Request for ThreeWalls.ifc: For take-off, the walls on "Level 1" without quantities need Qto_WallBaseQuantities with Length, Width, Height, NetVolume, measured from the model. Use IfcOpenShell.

First a look at what the model holds.

```python
import ifcopenshell
import ifcopenshell.util.element
import ifcopenshell.util.unit

model = ifcopenshell.open("ThreeWalls.ifc")
print(model.schema)
for unit_type in ("LENGTHUNIT", "AREAUNIT", "VOLUMEUNIT"):
    print(unit_type, ifcopenshell.util.unit.calculate_unit_scale(model, unit_type))
storey = next(s for s in model.by_type("IfcBuildingStorey") if s.Name == "Level 1")
walls = [e for e in ifcopenshell.util.element.get_decomposition(storey) if e.is_a("IfcWall")]
for e in sorted(walls, key=lambda e: e.id()):
    print(e.id(), e.is_a(), e.Name, list(ifcopenshell.util.element.get_psets(e, qtos_only=True)), sep=" | ")
```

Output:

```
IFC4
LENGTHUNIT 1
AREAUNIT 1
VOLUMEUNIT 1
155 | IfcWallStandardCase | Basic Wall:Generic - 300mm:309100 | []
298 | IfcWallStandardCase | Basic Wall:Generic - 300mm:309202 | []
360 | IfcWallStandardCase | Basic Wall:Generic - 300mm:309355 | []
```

```python
import ifcopenshell
import ifcopenshell.api.pset
import ifcopenshell.geom
import ifcopenshell.util.element
import ifcopenshell.util.shape
import ifcopenshell.util.unit

model = ifcopenshell.open("ThreeWalls.ifc")
unit_scale = ifcopenshell.util.unit.calculate_unit_scale(model)
volume_scale = ifcopenshell.util.unit.calculate_unit_scale(model, "VOLUMEUNIT")
settings = ifcopenshell.geom.settings()

storey = next(s for s in model.by_type("IfcBuildingStorey") if s.Name == "Level 1")
walls = [e for e in ifcopenshell.util.element.get_decomposition(storey) if e.is_a("IfcWall")]

for e in sorted(walls, key=lambda e: e.id()):
    if ifcopenshell.util.element.get_psets(e, qtos_only=True, should_inherit=False):
        continue
    # Geometry comes back in metres, in the element's own axes.
    shape = ifcopenshell.geom.create_shape(settings, e)
    values = {
        "Length": ifcopenshell.util.shape.get_x(shape.geometry) / unit_scale,
        "Width": ifcopenshell.util.shape.get_y(shape.geometry) / unit_scale,
        "Height": ifcopenshell.util.shape.get_z(shape.geometry) / unit_scale,
        "NetVolume": ifcopenshell.util.shape.get_volume(shape.geometry) / volume_scale,
    }
    qto = ifcopenshell.api.pset.add_qto(model, product=e, name="Qto_WallBaseQuantities")
    ifcopenshell.api.pset.edit_qto(model, qto=qto, properties=values)
    print(e.id(), {k: round(v, 3) for k, v in values.items()})

model.write("ThreeWalls_edited.ifc")
```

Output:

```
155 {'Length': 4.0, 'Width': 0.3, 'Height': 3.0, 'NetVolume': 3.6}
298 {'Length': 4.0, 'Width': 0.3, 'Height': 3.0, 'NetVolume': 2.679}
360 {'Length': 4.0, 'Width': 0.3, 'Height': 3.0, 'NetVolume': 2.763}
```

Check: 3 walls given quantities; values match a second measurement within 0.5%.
